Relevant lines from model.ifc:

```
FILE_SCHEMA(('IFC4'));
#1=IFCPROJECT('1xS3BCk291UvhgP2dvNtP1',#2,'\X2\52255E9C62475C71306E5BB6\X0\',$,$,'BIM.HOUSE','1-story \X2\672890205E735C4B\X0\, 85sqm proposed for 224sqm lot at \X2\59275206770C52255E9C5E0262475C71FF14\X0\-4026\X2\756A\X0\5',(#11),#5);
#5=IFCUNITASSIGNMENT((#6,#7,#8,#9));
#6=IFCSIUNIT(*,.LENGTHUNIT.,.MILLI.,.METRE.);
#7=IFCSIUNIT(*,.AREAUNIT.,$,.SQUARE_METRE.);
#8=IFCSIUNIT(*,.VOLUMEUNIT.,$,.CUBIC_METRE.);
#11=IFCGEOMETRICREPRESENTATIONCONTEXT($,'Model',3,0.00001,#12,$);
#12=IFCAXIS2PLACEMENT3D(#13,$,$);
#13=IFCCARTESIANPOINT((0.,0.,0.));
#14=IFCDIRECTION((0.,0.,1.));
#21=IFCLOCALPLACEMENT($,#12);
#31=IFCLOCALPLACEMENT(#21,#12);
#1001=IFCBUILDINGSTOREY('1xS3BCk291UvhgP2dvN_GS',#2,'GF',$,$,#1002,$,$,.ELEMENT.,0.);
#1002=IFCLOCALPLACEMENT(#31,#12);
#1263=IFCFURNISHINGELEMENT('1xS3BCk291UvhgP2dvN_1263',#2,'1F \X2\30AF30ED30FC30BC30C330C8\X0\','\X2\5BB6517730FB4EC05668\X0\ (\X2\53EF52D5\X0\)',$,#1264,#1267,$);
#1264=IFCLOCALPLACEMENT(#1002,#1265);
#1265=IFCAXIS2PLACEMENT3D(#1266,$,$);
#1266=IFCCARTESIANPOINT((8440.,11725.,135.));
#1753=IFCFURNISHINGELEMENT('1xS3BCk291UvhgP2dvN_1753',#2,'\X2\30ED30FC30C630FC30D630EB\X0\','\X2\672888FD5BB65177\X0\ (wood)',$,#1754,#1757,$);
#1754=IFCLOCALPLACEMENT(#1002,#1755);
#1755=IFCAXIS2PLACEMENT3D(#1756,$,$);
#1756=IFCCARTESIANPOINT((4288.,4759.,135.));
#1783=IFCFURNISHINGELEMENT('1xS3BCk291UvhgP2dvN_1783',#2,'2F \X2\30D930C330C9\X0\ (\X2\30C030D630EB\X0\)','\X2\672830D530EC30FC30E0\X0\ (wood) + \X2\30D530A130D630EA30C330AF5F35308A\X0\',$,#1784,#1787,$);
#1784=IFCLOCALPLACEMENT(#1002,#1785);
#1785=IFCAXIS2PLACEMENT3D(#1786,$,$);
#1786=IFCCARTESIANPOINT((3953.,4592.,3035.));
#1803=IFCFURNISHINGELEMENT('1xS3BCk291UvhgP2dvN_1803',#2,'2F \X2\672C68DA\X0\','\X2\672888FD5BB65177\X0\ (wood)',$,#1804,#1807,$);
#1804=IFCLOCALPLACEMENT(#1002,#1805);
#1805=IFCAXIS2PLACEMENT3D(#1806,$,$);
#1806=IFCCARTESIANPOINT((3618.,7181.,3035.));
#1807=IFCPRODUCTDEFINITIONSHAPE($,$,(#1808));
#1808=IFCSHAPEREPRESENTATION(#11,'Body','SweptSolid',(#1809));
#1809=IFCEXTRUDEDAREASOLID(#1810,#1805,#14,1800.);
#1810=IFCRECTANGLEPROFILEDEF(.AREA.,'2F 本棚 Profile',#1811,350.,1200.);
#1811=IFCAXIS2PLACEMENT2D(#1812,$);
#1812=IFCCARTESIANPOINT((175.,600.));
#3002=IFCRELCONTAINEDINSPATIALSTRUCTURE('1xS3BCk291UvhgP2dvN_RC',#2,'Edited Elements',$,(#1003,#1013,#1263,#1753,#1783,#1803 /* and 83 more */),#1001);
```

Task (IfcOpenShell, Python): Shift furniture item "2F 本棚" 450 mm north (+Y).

```python
import ifcopenshell
import ifcopenshell.api.geometry
import ifcopenshell.util.placement
import ifcopenshell.util.unit

model = ifcopenshell.open("model.ifc")
unit_scale = ifcopenshell.util.unit.calculate_unit_scale(model)

item = model.by_id(1803)
matrix = ifcopenshell.util.placement.get_local_placement(item.ObjectPlacement)
matrix[1, 3] += 0.45 / unit_scale
ifcopenshell.api.geometry.edit_object_placement(model, product=item, matrix=matrix, is_si=False)

print(ifcopenshell.util.placement.get_local_placement(item.ObjectPlacement).round(3) + 0.0)

model.write("model_rev.ifc")
```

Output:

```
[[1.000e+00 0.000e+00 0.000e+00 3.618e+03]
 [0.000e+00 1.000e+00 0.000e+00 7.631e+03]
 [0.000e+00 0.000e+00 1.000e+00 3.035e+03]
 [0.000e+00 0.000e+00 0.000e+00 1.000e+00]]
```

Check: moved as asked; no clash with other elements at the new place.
